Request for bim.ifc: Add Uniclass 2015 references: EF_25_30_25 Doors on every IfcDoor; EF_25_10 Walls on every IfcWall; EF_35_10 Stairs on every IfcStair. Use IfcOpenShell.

First a look at what the model holds.

```python
import ifcopenshell

model = ifcopenshell.open("bim.ifc")
print(model.schema)
print("classifications:", [c.Name for c in model.by_type("IfcClassification")])
for ifc_class in ("IfcDoor", "IfcRoof", "IfcStair", "IfcWall", "IfcWindow"):
    print(ifc_class, len(model.by_type(ifc_class)))
```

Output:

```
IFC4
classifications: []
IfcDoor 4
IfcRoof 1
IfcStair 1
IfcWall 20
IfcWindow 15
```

```python
import ifcopenshell
import ifcopenshell.api.classification

model = ifcopenshell.open("bim.ifc")

system = ifcopenshell.api.classification.add_classification(model, classification="Uniclass 2015")

codes = {
    "IfcDoor": ("EF_25_30_25", "Doors"),
    "IfcWall": ("EF_25_10", "Walls"),
    "IfcStair": ("EF_35_10", "Stairs"),
}
for ifc_class, (code, name) in codes.items():
    products = model.by_type(ifc_class)
    ifcopenshell.api.classification.add_reference(
        model, products=products, classification=system, identification=code, name=name
    )
    print(code, len(products))

model.write("bim_edited.ifc")
```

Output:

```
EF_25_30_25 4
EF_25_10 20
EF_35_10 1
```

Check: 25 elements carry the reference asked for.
